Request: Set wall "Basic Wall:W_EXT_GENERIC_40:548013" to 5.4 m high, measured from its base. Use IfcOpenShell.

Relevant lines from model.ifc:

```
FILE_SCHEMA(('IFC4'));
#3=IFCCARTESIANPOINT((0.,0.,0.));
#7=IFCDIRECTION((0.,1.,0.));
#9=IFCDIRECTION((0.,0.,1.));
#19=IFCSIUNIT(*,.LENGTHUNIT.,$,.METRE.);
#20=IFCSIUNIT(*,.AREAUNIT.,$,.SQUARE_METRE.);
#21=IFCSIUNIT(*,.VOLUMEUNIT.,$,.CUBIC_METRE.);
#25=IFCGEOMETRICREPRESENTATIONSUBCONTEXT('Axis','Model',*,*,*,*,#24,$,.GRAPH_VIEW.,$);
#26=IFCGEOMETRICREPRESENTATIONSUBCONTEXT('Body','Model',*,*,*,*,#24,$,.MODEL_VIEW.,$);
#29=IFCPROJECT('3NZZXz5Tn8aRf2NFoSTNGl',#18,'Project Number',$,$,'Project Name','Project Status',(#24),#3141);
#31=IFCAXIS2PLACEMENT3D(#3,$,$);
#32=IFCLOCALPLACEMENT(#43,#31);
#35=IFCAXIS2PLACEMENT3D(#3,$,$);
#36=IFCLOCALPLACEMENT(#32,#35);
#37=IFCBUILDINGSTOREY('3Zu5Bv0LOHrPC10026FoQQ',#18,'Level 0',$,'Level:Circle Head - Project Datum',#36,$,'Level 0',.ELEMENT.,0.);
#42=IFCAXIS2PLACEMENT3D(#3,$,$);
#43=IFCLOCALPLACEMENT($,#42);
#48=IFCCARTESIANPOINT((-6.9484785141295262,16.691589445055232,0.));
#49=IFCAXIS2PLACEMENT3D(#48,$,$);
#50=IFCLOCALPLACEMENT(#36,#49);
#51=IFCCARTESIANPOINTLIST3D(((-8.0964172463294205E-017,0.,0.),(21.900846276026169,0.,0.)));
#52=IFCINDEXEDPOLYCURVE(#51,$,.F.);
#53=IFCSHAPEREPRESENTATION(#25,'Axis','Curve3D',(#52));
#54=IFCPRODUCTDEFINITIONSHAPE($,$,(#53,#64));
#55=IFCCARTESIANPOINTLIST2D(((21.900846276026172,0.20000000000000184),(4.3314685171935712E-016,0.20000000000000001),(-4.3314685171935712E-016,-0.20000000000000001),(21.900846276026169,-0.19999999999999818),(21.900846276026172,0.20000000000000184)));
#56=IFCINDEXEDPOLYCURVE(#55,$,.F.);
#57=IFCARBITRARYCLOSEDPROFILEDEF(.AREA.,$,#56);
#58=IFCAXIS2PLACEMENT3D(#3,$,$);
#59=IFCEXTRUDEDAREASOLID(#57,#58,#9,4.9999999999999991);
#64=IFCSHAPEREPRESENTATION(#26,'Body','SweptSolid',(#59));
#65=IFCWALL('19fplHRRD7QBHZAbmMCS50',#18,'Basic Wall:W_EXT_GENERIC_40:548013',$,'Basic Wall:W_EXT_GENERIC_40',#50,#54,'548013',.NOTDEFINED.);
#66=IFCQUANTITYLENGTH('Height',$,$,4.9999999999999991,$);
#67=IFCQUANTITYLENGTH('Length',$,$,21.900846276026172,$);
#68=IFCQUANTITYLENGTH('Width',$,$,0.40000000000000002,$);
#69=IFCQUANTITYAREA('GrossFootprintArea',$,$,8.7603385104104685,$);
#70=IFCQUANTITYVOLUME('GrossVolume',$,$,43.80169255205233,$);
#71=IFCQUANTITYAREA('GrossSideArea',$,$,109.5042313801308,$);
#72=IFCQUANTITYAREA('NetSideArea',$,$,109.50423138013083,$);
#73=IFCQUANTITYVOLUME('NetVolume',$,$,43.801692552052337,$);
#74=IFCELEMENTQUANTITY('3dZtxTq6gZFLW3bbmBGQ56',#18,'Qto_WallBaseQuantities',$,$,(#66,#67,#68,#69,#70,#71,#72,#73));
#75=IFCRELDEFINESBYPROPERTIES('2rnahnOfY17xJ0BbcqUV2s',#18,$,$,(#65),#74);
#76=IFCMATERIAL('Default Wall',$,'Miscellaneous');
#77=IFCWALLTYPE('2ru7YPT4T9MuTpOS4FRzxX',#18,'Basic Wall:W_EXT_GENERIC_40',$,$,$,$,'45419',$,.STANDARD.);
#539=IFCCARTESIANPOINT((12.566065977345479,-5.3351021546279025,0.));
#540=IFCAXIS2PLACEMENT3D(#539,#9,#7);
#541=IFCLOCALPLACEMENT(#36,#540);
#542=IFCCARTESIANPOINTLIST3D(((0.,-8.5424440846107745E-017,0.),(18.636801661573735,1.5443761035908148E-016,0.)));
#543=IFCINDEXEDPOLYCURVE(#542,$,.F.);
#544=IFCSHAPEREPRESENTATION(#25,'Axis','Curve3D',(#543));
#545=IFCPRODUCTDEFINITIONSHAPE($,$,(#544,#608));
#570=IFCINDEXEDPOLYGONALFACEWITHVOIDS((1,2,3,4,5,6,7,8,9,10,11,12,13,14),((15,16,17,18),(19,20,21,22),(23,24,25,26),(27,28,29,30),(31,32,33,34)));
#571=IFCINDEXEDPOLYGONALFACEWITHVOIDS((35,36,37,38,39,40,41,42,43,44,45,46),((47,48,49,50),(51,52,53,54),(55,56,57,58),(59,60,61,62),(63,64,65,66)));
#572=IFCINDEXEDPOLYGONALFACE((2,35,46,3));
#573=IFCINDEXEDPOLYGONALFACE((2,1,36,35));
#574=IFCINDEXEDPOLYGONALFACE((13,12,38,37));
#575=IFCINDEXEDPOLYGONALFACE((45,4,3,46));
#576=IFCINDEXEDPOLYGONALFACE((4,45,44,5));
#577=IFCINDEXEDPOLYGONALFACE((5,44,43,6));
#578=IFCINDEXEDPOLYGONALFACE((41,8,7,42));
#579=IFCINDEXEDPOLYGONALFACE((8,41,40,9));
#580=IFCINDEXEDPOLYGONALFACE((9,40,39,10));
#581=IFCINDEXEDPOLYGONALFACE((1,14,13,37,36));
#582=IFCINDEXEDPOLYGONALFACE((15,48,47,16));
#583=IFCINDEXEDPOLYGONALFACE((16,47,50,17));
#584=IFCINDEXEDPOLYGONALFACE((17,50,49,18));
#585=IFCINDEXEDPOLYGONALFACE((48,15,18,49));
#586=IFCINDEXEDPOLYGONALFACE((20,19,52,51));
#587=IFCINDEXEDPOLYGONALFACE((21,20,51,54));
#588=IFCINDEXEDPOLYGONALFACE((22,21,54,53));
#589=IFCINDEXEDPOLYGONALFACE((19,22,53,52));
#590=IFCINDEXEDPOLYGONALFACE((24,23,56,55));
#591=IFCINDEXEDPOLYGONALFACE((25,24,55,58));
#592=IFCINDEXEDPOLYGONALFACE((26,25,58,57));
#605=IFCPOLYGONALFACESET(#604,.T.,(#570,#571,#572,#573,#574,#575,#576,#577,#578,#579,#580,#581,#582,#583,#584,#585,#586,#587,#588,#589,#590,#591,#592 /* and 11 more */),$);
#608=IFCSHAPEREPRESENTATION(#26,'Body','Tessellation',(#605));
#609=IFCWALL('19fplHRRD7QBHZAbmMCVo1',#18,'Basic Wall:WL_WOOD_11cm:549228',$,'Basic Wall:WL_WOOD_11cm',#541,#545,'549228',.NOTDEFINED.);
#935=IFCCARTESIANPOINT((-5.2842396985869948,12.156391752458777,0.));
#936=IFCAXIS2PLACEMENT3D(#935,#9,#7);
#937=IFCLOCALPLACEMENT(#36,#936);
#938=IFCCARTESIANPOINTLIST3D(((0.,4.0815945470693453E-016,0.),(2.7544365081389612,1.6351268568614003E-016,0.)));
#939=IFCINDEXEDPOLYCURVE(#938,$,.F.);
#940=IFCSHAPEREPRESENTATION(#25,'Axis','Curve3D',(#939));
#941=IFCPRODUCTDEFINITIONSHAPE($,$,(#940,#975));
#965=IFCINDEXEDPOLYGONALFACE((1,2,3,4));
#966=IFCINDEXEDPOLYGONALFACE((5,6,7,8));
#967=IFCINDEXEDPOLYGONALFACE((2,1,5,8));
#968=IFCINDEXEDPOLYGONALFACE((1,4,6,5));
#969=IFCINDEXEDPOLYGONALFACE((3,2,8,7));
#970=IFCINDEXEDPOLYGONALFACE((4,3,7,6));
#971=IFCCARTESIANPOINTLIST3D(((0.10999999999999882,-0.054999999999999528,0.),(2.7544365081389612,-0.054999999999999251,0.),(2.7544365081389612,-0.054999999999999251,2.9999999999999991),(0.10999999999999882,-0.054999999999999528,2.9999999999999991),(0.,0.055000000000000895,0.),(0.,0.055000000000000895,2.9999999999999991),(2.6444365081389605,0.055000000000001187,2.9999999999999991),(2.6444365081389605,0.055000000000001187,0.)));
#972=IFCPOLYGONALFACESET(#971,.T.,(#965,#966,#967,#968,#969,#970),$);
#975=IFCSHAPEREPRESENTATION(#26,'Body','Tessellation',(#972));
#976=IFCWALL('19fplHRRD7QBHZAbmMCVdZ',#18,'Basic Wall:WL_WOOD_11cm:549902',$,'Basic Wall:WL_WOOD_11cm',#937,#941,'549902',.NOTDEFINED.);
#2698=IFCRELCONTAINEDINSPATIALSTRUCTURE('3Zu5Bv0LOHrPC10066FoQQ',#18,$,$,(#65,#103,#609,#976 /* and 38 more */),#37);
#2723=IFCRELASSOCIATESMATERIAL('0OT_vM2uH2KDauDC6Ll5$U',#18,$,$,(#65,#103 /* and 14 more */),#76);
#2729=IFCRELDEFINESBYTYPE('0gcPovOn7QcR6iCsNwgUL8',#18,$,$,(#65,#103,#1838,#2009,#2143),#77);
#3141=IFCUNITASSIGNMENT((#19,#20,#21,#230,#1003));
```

```python
import ifcopenshell
import ifcopenshell.api.pset
import ifcopenshell.geom
import ifcopenshell.util.element
import ifcopenshell.util.representation
import ifcopenshell.util.shape
import ifcopenshell.util.unit

model = ifcopenshell.open("model.ifc")
unit_scale = ifcopenshell.util.unit.calculate_unit_scale(model)
area_scale = ifcopenshell.util.unit.calculate_unit_scale(model, "AREAUNIT")
volume_scale = ifcopenshell.util.unit.calculate_unit_scale(model, "VOLUMEUNIT")
settings = ifcopenshell.geom.settings()


def volume(element):
    """Net volume in cubic metres, openings subtracted."""
    shape = ifcopenshell.geom.create_shape(settings, element)
    return ifcopenshell.util.shape.get_volume(shape.geometry)


wall = model.by_guid("19fplHRRD7QBHZAbmMCS50")
before = volume(wall)

body = ifcopenshell.util.representation.get_representation(wall, "Model", "Body")
solid = body.Items[0]
old_height = solid.Depth
solid.Depth = 5.4
after = volume(wall)
thickness = 0.4  # wall thickness in metres

# Update the stored height, areas and volumes.
qto = model.by_id(ifcopenshell.util.element.get_pset(wall, "Qto_WallBaseQuantities", should_inherit=False)["id"])
ifcopenshell.api.pset.edit_qto(model, qto=qto, properties={
    "Height": solid.Depth,
    "GrossVolume": ifcopenshell.util.element.get_pset(wall, "Qto_WallBaseQuantities", "GrossVolume") * solid.Depth / old_height,
    "GrossSideArea": ifcopenshell.util.element.get_pset(wall, "Qto_WallBaseQuantities", "GrossSideArea") * solid.Depth / old_height,
    "NetSideArea": after / thickness / area_scale,
    "NetVolume": after / volume_scale,
})

print(f"height {old_height:g} -> {solid.Depth:g}, volume {before:.3f} -> {after:.3f} m3")

model.write("model-out.ifc")
```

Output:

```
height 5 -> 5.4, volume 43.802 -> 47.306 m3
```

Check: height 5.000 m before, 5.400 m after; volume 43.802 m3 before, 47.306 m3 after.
